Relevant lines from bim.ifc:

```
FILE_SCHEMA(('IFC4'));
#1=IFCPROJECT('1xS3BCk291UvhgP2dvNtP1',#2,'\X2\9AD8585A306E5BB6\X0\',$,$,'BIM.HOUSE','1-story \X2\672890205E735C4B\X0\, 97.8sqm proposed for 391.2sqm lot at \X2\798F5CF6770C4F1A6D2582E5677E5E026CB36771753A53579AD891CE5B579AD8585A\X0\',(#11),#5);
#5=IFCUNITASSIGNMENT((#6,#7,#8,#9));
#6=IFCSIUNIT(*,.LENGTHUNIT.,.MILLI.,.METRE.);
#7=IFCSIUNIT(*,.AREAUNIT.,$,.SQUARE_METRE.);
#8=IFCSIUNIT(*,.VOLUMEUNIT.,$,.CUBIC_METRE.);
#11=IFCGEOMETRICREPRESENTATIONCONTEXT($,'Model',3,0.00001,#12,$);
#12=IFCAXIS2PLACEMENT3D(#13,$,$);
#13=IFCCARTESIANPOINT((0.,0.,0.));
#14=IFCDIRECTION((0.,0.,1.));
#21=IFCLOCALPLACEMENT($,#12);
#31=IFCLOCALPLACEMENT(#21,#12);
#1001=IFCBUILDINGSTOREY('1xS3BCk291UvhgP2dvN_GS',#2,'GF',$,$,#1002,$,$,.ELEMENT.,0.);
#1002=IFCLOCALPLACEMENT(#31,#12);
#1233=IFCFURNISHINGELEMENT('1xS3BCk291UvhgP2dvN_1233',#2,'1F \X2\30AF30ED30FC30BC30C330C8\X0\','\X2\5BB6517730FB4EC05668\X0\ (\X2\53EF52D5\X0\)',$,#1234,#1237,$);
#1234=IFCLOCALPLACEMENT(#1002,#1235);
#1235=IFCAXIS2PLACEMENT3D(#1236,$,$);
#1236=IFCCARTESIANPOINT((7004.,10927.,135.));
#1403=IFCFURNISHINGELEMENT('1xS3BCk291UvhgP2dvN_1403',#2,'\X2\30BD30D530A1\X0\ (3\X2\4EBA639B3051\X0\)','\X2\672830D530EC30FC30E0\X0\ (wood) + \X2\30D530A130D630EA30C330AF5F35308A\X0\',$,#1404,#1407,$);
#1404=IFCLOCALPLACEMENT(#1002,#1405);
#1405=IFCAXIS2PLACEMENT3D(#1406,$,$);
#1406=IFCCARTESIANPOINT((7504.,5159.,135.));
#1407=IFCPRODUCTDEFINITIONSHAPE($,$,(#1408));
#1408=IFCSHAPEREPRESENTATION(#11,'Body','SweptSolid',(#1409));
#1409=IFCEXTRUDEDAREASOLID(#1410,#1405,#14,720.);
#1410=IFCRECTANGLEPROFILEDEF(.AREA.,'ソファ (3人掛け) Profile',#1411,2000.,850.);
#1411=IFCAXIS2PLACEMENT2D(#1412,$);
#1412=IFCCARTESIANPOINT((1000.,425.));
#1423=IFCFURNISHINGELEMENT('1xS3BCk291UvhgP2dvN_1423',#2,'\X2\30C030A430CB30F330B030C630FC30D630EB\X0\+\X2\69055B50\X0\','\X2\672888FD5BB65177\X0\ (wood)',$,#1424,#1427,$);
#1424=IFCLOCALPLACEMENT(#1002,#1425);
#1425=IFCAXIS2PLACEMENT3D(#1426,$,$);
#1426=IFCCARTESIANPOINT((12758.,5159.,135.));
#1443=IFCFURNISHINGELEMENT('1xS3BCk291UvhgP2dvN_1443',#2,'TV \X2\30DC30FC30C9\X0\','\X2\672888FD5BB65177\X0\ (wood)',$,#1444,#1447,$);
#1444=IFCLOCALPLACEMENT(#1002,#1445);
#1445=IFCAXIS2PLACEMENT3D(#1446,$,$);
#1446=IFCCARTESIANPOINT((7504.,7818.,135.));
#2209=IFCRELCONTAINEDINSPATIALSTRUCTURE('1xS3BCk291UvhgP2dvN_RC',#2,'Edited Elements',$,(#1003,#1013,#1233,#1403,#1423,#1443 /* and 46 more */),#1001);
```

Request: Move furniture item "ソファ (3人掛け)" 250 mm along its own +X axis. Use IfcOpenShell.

```python
import ifcopenshell
import ifcopenshell.api.geometry
import ifcopenshell.util.placement
import ifcopenshell.util.unit

model = ifcopenshell.open("bim.ifc")
unit_scale = ifcopenshell.util.unit.calculate_unit_scale(model)

item = model.by_guid("1xS3BCk291UvhgP2dvN_1403")
matrix = ifcopenshell.util.placement.get_local_placement(item.ObjectPlacement)
matrix[:3, 3] += matrix[:3, 0] * 0.25 / unit_scale
ifcopenshell.api.geometry.edit_object_placement(model, product=item, matrix=matrix, is_si=False)

print(ifcopenshell.util.placement.get_local_placement(item.ObjectPlacement).round(3) + 0.0)

model.write("bim_rev.ifc")
```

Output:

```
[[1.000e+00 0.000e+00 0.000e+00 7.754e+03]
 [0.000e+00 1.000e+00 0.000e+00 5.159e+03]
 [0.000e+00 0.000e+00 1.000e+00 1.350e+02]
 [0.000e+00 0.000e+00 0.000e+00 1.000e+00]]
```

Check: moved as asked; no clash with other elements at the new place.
